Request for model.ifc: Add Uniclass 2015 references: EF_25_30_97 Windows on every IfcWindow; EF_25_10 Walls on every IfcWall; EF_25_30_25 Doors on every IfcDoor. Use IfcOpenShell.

First a look at what the model holds.

```python
import ifcopenshell

model = ifcopenshell.open("model.ifc")
print(model.schema)
print("classifications:", [c.Name for c in model.by_type("IfcClassification")])
for ifc_class in ("IfcDoor", "IfcRoof", "IfcStair", "IfcWall", "IfcWindow"):
    print(ifc_class, len(model.by_type(ifc_class)))
```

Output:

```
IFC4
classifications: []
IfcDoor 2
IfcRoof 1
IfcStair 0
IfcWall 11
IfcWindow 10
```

```python
import ifcopenshell
import ifcopenshell.api.classification

model = ifcopenshell.open("model.ifc")

system = ifcopenshell.api.classification.add_classification(model, classification="Uniclass 2015")

codes = {
    "IfcWindow": ("EF_25_30_97", "Windows"),
    "IfcWall": ("EF_25_10", "Walls"),
    "IfcDoor": ("EF_25_30_25", "Doors"),
}
for ifc_class, (code, name) in codes.items():
    products = model.by_type(ifc_class)
    ifcopenshell.api.classification.add_reference(
        model, products=products, classification=system, identification=code, name=name
    )
    print(code, len(products))

model.write("model_edited.ifc")
```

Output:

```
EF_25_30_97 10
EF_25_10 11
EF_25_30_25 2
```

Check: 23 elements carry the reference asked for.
